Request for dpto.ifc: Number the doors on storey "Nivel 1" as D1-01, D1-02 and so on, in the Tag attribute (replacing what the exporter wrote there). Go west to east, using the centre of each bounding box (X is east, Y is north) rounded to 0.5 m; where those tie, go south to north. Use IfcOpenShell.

First a look at what the model holds.

```python
import ifcopenshell
import ifcopenshell.util.element
import ifcopenshell.util.placement

model = ifcopenshell.open("dpto.ifc")
print(model.schema)
storey = next(s for s in model.by_type("IfcBuildingStorey") if s.Name == "Nivel 1")
doors = [e for e in ifcopenshell.util.element.get_decomposition(storey) if e.is_a("IfcDoor")]
for e in sorted(doors, key=lambda e: e.id()):
    origin = ifcopenshell.util.placement.get_local_placement(e.ObjectPlacement)[:3, 3]
    print(e.id(), e.Tag, e.Name, origin.round(2) + 0.0, sep=" | ")
```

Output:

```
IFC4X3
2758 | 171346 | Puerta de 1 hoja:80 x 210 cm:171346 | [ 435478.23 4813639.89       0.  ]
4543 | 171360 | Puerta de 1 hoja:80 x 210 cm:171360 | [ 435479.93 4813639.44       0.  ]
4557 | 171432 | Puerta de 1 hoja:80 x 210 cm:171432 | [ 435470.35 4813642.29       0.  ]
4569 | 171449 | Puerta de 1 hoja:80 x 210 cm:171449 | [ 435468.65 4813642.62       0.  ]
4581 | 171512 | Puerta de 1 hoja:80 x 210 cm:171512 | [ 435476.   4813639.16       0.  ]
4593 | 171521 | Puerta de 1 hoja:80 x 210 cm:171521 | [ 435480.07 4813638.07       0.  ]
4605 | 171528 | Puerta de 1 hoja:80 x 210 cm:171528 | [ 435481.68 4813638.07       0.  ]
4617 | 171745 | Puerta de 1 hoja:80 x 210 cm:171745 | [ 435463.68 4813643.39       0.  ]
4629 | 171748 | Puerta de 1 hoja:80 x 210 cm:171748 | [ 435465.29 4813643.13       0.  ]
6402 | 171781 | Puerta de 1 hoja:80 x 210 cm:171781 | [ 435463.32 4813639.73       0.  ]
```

```python
import ifcopenshell
import ifcopenshell.geom
import ifcopenshell.util.element
import ifcopenshell.util.shape

model = ifcopenshell.open("dpto.ifc")
settings = ifcopenshell.geom.settings()
settings.set("use-world-coords", True)


def centre(element):
    shape = ifcopenshell.geom.create_shape(settings, element)
    return ifcopenshell.util.shape.get_bbox_centroid(shape.geometry)


storey = next(s for s in model.by_type("IfcBuildingStorey") if s.Name == "Nivel 1")
doors = [e for e in ifcopenshell.util.element.get_decomposition(storey) if e.is_a("IfcDoor")]

# Insertion points can sit at a corner or the storey origin, so sort by the geometry (in metres).
centres = {e: centre(e) for e in doors}
doors.sort(key=lambda e: (round(centres[e][0] / 0.5), centres[e][1]))

for i, e in enumerate(doors, start=1):
    number = f"D1-{i:02d}"
    e.Tag = number
    print(e.id(), number)

model.write("dpto_edited.ifc")
```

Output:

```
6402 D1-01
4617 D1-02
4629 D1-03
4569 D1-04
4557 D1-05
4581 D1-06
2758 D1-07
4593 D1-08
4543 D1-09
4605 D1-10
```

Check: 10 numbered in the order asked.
